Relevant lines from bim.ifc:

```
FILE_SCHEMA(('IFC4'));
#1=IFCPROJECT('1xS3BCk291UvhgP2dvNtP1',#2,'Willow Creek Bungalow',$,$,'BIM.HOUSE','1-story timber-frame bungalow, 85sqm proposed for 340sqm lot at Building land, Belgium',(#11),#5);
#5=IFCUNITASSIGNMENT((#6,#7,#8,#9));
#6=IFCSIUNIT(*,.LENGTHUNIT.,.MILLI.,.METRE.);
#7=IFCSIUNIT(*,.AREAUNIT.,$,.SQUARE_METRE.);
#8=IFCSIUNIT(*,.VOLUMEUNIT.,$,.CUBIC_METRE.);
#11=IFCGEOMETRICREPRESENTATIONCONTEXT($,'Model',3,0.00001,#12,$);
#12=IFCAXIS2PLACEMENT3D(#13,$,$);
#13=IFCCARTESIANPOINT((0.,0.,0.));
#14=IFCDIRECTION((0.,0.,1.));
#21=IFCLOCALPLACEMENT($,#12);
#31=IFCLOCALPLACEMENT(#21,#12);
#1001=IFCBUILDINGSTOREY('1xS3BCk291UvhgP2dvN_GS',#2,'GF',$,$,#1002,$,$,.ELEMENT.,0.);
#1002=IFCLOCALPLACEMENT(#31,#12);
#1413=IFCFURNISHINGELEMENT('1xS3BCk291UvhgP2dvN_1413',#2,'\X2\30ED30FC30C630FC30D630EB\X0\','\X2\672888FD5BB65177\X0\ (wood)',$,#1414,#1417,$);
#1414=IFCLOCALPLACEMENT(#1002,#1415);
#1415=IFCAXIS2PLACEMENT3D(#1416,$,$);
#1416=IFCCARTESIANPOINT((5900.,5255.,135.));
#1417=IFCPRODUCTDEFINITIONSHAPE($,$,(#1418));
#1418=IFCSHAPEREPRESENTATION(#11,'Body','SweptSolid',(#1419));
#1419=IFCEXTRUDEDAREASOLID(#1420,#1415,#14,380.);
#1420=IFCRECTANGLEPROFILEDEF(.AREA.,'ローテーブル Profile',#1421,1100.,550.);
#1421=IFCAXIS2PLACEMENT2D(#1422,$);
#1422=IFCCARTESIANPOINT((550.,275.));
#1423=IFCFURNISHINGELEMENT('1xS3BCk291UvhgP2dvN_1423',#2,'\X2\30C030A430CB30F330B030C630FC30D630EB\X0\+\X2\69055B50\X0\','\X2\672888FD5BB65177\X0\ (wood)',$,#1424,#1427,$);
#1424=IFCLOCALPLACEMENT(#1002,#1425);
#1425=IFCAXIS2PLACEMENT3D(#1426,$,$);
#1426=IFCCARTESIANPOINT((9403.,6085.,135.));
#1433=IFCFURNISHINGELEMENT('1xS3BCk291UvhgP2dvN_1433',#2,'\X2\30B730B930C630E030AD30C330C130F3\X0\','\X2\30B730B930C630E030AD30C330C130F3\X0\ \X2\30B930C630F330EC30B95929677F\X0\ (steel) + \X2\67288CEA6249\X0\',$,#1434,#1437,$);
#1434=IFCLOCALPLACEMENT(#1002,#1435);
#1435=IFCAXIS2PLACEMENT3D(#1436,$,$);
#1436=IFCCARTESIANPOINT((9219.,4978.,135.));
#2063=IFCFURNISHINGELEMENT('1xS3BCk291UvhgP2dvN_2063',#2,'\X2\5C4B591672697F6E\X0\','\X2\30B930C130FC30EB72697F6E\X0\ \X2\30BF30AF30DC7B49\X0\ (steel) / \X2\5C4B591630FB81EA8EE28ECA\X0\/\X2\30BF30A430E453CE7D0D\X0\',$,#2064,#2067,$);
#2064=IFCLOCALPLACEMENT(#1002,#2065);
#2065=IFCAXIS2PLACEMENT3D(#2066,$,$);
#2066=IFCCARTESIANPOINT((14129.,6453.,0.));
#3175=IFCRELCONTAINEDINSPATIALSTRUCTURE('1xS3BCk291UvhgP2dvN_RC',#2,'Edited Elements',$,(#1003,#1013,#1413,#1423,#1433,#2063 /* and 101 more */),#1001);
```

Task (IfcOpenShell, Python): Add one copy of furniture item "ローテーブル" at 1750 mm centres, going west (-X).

```python
import numpy as np
import ifcopenshell
import ifcopenshell.api.geometry
import ifcopenshell.api.root
import ifcopenshell.util.element
import ifcopenshell.util.placement
import ifcopenshell.util.unit

model = ifcopenshell.open("bim.ifc")
unit_scale = ifcopenshell.util.unit.calculate_unit_scale(model)


def reuse_history(source, copy):
    """copy_class also copies each property set's owner history, people and application; keep the originals."""
    for rel in copy.IsDefinedBy:
        if rel.is_a("IfcRelDefinesByProperties") and (history := rel.RelatingPropertyDefinition.OwnerHistory):
            rel.RelatingPropertyDefinition.OwnerHistory = source.OwnerHistory
            ifcopenshell.util.element.remove_deep2(model, history)


source = model.by_id(1413)
base = ifcopenshell.util.placement.get_local_placement(source.ObjectPlacement)
step = np.array([-1.0, 0.0, 0.0]) * 1.75 / unit_scale

for i in range(1, 2):
    copy = ifcopenshell.api.root.copy_class(model, product=source)
    copy.Representation = ifcopenshell.util.element.copy_deep(
        model, source.Representation, exclude=["IfcGeometricRepresentationContext", "IfcRepresentationMap"]
    )
    reuse_history(source, copy)
    matrix = base.copy()
    matrix[:3, 3] += i * step
    print("added at", matrix[:3, 3].round(3) + 0.0)
    ifcopenshell.api.geometry.edit_object_placement(model, product=copy, matrix=matrix, is_si=False)

model.write("bim_edited.ifc")
```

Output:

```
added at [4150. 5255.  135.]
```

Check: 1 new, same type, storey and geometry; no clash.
